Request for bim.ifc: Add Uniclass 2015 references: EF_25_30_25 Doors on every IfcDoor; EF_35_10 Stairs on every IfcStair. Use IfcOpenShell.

First a look at what the model holds.

```python
import ifcopenshell

model = ifcopenshell.open("bim.ifc")
print(model.schema)
print("classifications:", [c.Name for c in model.by_type("IfcClassification")])
for ifc_class in ("IfcDoor", "IfcRoof", "IfcStair", "IfcWall", "IfcWindow"):
    print(ifc_class, len(model.by_type(ifc_class)))
```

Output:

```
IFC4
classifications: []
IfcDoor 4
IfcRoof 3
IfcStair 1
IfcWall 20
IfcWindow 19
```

```python
import ifcopenshell
import ifcopenshell.api.classification

model = ifcopenshell.open("bim.ifc")

system = ifcopenshell.api.classification.add_classification(model, classification="Uniclass 2015")

codes = {
    "IfcDoor": ("EF_25_30_25", "Doors"),
    "IfcStair": ("EF_35_10", "Stairs"),
}
for ifc_class, (code, name) in codes.items():
    products = model.by_type(ifc_class)
    ifcopenshell.api.classification.add_reference(
        model, products=products, classification=system, identification=code, name=name
    )
    print(code, len(products))

model.write("bim_rev.ifc")
```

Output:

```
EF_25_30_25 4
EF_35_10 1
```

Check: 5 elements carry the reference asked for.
